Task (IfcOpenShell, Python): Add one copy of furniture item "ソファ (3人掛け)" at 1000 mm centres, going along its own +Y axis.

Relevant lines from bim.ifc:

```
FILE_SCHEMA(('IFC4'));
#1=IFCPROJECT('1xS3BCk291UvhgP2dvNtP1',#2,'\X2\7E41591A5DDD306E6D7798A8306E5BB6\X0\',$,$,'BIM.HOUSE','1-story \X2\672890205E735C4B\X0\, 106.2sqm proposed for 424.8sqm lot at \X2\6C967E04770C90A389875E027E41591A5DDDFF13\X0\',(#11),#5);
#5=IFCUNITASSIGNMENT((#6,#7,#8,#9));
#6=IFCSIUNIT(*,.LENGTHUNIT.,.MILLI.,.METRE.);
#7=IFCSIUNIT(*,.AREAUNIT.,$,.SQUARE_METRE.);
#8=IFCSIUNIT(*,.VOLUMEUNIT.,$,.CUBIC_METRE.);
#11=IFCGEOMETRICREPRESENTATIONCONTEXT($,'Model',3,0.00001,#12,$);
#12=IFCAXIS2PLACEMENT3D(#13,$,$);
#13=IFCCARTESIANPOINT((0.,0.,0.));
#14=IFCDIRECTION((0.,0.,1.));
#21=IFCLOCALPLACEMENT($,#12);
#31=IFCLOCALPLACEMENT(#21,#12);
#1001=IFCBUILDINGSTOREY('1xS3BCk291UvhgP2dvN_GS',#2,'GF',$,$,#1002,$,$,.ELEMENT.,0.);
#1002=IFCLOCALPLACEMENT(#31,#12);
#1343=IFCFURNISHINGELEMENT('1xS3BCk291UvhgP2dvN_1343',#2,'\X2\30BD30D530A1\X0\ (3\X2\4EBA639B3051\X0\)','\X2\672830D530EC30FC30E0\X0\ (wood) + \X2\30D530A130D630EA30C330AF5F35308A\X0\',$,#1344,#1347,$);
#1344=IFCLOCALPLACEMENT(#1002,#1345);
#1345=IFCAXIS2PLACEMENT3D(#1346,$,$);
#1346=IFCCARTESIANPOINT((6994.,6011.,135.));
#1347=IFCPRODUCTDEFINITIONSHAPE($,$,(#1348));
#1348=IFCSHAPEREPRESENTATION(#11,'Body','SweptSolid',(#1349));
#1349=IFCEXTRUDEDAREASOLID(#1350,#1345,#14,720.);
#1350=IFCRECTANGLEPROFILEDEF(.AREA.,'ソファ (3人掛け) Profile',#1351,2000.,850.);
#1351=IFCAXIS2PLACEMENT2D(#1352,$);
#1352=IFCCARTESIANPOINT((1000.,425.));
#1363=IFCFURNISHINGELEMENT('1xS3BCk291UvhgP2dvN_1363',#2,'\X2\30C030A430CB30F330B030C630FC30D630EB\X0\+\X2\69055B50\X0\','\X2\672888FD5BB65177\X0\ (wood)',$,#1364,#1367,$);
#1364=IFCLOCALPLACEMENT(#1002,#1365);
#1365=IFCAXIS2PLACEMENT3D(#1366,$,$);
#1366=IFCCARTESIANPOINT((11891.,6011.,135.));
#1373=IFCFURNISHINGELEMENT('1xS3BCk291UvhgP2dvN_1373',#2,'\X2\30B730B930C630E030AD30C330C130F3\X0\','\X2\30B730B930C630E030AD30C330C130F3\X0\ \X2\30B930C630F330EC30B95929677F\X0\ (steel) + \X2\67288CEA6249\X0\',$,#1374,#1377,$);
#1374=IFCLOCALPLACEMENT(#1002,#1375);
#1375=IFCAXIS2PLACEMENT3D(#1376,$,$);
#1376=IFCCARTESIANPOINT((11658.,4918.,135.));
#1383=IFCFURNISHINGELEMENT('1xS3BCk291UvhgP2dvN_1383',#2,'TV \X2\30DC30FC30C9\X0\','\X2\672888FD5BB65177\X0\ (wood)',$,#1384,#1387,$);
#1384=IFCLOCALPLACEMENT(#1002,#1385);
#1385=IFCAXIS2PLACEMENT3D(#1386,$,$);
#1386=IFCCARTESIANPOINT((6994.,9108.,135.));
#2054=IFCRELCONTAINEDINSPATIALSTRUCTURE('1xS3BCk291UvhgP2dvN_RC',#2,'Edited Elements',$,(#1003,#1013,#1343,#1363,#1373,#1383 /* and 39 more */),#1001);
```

```python
import ifcopenshell
import ifcopenshell.api.geometry
import ifcopenshell.api.root
import ifcopenshell.util.element
import ifcopenshell.util.placement
import ifcopenshell.util.unit

model = ifcopenshell.open("bim.ifc")
unit_scale = ifcopenshell.util.unit.calculate_unit_scale(model)


def reuse_history(source, copy):
    """copy_class also copies each property set's owner history, people and application; keep the originals."""
    for rel in copy.IsDefinedBy:
        if rel.is_a("IfcRelDefinesByProperties") and (history := rel.RelatingPropertyDefinition.OwnerHistory):
            rel.RelatingPropertyDefinition.OwnerHistory = source.OwnerHistory
            ifcopenshell.util.element.remove_deep2(model, history)


source = model.by_guid("1xS3BCk291UvhgP2dvN_1343")
base = ifcopenshell.util.placement.get_local_placement(source.ObjectPlacement)
step = base[:3, 1] * 1 / unit_scale

for i in range(1, 2):
    copy = ifcopenshell.api.root.copy_class(model, product=source)
    copy.Representation = ifcopenshell.util.element.copy_deep(
        model, source.Representation, exclude=["IfcGeometricRepresentationContext", "IfcRepresentationMap"]
    )
    reuse_history(source, copy)
    matrix = base.copy()
    matrix[:3, 3] += i * step
    print("added at", matrix[:3, 3].round(3) + 0.0)
    ifcopenshell.api.geometry.edit_object_placement(model, product=copy, matrix=matrix, is_si=False)

model.write("bim_edited.ifc")
```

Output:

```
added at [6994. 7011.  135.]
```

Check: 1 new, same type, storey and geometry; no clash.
